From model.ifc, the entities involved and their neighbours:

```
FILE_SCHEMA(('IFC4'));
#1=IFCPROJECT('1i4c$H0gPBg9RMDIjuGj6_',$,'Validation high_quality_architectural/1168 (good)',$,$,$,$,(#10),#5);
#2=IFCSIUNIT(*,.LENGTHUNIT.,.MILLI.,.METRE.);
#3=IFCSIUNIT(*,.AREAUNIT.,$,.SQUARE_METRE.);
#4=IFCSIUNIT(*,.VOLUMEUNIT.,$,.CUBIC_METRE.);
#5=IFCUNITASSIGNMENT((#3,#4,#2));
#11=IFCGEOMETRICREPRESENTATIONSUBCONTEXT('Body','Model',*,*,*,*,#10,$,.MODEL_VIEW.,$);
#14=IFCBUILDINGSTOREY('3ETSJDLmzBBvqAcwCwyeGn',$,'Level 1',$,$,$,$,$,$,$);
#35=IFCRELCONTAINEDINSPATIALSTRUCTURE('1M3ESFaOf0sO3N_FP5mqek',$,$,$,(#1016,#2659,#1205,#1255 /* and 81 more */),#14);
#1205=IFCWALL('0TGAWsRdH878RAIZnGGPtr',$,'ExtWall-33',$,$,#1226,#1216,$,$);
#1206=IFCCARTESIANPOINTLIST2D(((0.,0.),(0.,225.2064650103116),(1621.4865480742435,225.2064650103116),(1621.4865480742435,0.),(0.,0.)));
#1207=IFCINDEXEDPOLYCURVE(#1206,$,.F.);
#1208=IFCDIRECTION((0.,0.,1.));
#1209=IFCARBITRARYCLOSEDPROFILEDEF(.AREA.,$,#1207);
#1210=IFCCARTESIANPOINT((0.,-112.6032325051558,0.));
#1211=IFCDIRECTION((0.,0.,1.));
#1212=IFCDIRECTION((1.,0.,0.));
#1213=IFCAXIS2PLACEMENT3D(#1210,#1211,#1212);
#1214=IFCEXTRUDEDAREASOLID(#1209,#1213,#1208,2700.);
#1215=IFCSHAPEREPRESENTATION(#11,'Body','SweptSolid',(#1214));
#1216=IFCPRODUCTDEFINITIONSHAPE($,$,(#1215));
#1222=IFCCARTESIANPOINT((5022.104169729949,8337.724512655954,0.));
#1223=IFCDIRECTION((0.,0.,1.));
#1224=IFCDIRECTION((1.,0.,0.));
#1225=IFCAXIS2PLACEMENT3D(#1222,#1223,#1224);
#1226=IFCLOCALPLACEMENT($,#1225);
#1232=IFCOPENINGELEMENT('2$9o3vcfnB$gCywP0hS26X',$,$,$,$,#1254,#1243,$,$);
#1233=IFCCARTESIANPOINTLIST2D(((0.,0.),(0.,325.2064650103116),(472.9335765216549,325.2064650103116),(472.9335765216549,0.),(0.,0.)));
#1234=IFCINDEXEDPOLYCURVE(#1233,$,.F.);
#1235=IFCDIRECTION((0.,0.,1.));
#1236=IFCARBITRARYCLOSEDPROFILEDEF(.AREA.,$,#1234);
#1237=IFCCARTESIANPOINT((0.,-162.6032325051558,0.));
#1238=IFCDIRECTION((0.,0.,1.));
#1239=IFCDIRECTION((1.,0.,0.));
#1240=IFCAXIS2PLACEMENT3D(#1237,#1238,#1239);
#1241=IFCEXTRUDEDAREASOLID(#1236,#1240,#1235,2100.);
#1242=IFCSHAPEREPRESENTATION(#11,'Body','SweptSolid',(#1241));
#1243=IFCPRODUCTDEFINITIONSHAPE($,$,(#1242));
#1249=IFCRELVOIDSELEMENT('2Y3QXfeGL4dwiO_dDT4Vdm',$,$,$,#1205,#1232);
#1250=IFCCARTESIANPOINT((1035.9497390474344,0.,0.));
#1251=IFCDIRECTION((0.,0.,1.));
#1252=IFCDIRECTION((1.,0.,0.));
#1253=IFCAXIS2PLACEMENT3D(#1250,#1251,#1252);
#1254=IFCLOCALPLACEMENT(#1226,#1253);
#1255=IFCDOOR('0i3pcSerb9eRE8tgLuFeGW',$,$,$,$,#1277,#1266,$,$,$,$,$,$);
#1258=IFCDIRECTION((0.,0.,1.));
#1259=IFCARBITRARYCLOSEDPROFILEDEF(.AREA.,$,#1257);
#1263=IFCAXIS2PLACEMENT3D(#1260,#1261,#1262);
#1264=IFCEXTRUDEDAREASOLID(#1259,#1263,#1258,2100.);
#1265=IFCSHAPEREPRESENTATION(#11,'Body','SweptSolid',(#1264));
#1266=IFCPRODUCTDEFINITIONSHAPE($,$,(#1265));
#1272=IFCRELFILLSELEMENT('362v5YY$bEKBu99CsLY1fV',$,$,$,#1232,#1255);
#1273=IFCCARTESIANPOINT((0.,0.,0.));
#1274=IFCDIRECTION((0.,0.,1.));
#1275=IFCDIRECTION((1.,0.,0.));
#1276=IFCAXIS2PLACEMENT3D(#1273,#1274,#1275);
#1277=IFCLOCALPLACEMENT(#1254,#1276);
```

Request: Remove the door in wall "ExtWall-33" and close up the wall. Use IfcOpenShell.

```python
import ifcopenshell
import ifcopenshell.api.feature
import ifcopenshell.api.root
import ifcopenshell.geom
import ifcopenshell.util.shape

model = ifcopenshell.open("model.ifc")
settings = ifcopenshell.geom.settings()


def volume(element):
    """Net volume in cubic metres, openings subtracted."""
    shape = ifcopenshell.geom.create_shape(settings, element)
    return ifcopenshell.util.shape.get_volume(shape.geometry)


door = model.by_id(1255)
opening = door.FillsVoids[0].RelatingOpeningElement
wall = opening.VoidsElements[0].RelatingBuildingElement
before = volume(wall)

ifcopenshell.api.root.remove_product(model, product=door)
ifcopenshell.api.feature.remove_feature(model, feature=opening)

after = volume(wall)

print(f"wall volume {before:.3f} -> {after:.3f} m3")

model.write("model_updated.ifc")
```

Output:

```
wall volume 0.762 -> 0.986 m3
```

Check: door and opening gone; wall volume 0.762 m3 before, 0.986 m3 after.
